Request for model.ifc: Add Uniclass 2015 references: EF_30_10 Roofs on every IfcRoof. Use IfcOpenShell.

First a look at what the model holds.

```python
import ifcopenshell

model = ifcopenshell.open("model.ifc")
print(model.schema)
print("classifications:", [c.Name for c in model.by_type("IfcClassification")])
for ifc_class in ("IfcDoor", "IfcRoof", "IfcStair", "IfcWall", "IfcWindow"):
    print(ifc_class, len(model.by_type(ifc_class)))
```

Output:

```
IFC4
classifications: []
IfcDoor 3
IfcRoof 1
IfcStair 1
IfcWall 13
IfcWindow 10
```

```python
import ifcopenshell
import ifcopenshell.api.classification

model = ifcopenshell.open("model.ifc")

system = ifcopenshell.api.classification.add_classification(model, classification="Uniclass 2015")

codes = {
    "IfcRoof": ("EF_30_10", "Roofs"),
}
for ifc_class, (code, name) in codes.items():
    products = model.by_type(ifc_class)
    ifcopenshell.api.classification.add_reference(
        model, products=products, classification=system, identification=code, name=name
    )
    print(code, len(products))

model.write("model_rev.ifc")
```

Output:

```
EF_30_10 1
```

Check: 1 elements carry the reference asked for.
